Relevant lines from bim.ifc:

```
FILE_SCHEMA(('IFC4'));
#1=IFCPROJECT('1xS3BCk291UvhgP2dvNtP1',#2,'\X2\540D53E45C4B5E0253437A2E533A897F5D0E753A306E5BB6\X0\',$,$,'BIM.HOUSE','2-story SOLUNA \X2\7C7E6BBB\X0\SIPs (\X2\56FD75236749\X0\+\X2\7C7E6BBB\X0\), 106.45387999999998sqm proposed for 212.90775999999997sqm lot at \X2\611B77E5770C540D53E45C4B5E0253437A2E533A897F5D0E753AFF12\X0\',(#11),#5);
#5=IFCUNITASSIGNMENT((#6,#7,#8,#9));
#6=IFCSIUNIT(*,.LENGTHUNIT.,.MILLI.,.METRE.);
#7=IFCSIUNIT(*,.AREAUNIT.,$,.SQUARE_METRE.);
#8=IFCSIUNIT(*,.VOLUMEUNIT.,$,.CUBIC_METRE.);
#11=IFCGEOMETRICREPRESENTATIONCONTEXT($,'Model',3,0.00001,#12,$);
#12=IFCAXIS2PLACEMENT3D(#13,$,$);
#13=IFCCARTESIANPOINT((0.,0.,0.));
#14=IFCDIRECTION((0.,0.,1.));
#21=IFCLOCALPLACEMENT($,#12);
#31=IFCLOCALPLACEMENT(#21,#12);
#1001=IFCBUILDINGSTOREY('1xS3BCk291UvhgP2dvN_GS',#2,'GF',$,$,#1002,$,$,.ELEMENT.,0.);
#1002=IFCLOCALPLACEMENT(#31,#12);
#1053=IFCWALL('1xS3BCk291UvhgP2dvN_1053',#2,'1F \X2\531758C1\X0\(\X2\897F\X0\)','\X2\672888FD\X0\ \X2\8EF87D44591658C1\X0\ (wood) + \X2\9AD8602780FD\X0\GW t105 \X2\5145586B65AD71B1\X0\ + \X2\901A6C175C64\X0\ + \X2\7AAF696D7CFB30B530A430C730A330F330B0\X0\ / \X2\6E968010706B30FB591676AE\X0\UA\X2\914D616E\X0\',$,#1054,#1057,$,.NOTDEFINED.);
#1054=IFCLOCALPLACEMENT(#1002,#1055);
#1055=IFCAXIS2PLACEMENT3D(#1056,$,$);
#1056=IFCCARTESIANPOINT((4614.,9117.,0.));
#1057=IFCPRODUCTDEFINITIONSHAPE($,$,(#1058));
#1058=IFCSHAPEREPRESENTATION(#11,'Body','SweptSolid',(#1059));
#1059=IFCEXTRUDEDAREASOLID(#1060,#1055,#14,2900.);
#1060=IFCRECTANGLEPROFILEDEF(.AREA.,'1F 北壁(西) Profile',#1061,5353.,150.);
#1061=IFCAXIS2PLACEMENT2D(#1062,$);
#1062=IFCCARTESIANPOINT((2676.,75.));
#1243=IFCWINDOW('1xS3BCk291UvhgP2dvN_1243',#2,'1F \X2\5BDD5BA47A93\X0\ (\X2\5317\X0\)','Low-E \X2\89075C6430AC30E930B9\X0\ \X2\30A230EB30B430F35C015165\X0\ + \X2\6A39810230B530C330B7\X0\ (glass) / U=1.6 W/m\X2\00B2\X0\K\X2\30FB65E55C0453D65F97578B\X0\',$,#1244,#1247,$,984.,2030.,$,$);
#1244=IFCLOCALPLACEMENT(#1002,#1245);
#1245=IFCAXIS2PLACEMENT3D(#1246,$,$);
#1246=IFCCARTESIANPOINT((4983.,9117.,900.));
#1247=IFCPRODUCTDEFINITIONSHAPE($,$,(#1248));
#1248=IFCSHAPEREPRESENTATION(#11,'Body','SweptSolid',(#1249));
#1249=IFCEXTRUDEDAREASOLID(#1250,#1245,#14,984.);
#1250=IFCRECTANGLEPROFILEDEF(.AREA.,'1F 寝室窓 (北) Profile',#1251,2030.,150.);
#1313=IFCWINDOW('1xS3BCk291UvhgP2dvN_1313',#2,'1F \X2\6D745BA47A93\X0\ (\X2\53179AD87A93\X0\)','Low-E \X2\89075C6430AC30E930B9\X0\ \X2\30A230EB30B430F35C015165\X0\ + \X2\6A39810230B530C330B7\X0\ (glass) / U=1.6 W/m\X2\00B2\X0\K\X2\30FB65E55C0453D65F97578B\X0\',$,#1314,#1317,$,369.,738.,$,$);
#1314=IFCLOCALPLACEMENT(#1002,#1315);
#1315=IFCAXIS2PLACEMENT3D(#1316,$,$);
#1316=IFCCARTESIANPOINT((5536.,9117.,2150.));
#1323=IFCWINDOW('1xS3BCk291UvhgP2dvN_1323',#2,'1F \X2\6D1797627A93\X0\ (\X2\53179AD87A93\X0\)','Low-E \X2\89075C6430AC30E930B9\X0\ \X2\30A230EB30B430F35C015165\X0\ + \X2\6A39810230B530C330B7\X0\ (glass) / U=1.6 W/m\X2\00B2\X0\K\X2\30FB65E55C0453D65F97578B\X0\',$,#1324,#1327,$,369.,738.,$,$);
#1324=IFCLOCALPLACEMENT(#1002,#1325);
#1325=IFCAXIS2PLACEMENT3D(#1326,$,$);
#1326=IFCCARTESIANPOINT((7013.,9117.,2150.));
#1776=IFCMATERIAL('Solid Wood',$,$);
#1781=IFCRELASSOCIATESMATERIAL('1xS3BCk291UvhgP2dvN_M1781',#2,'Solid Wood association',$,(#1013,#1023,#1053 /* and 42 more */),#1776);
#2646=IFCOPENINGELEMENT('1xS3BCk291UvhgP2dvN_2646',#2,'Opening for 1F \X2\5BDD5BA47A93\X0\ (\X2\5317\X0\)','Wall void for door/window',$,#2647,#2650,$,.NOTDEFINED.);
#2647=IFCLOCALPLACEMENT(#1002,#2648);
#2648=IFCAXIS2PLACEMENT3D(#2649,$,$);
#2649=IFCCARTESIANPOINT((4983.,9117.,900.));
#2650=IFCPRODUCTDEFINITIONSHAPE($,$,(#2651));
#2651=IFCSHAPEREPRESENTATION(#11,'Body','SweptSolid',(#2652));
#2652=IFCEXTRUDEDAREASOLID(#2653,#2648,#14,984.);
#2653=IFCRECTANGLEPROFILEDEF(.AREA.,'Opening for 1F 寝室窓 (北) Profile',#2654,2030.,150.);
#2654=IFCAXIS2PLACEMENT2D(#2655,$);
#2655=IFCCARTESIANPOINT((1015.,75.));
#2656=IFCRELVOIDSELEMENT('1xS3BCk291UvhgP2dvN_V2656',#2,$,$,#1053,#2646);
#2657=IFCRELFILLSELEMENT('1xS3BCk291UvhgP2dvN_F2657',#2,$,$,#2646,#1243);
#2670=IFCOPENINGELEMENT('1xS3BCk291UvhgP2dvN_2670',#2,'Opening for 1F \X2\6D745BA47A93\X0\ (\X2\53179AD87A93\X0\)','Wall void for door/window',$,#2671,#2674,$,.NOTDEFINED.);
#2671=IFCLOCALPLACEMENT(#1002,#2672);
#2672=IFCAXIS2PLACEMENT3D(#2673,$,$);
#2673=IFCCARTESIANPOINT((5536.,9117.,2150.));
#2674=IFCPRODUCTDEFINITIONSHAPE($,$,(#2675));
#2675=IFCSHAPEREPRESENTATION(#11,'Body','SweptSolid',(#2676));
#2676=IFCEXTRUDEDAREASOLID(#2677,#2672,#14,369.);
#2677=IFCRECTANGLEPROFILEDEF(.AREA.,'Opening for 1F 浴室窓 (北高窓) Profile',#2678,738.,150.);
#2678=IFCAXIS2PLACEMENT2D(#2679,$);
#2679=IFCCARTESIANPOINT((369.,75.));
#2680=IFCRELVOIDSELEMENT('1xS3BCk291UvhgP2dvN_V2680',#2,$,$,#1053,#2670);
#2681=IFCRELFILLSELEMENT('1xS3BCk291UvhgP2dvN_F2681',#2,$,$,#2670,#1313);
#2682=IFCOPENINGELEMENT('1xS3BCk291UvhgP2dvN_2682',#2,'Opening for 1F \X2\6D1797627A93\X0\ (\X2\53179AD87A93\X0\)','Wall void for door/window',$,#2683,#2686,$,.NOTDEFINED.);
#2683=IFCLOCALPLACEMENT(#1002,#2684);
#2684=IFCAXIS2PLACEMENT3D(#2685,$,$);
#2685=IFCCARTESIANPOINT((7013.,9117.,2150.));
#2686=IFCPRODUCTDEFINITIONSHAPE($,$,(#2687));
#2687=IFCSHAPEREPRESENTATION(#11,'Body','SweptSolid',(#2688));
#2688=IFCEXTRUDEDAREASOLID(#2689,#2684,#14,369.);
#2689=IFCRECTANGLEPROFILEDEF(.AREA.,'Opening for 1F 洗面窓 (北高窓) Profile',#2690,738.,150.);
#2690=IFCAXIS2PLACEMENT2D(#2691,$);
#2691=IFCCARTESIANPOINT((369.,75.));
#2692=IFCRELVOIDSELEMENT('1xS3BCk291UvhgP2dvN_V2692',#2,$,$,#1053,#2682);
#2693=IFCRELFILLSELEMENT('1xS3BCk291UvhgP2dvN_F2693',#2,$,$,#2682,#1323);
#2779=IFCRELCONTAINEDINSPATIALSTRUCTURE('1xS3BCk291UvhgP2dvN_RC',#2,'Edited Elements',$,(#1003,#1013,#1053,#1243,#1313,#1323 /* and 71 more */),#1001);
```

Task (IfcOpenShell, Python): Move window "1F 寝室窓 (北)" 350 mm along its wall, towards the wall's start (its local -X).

```python
import ifcopenshell
import ifcopenshell.api.geometry
import ifcopenshell.util.placement
import ifcopenshell.util.unit

model = ifcopenshell.open("bim.ifc")
unit_scale = ifcopenshell.util.unit.calculate_unit_scale(model)

window = model.by_guid("1xS3BCk291UvhgP2dvN_1243")
opening = window.FillsVoids[0].RelatingOpeningElement
wall = opening.VoidsElements[0].RelatingBuildingElement

wall_matrix = ifcopenshell.util.placement.get_local_placement(wall.ObjectPlacement)
shift = wall_matrix[:3, 0] * -0.35 / unit_scale
before = ifcopenshell.util.placement.get_local_placement(window.ObjectPlacement)[:3, 3].copy()

# The window is not placed relative to its opening, so move both.
for product in (opening, window):
    matrix = ifcopenshell.util.placement.get_local_placement(product.ObjectPlacement)
    matrix[:3, 3] += shift
    ifcopenshell.api.geometry.edit_object_placement(model, product=product, matrix=matrix, is_si=False)

after = ifcopenshell.util.placement.get_local_placement(window.ObjectPlacement)[:3, 3]
print("window moved by", (after - before).round(3) + 0.0)

model.write("bim-out.ifc")
```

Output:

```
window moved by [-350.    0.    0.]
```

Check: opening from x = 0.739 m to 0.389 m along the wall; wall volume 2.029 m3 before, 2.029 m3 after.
